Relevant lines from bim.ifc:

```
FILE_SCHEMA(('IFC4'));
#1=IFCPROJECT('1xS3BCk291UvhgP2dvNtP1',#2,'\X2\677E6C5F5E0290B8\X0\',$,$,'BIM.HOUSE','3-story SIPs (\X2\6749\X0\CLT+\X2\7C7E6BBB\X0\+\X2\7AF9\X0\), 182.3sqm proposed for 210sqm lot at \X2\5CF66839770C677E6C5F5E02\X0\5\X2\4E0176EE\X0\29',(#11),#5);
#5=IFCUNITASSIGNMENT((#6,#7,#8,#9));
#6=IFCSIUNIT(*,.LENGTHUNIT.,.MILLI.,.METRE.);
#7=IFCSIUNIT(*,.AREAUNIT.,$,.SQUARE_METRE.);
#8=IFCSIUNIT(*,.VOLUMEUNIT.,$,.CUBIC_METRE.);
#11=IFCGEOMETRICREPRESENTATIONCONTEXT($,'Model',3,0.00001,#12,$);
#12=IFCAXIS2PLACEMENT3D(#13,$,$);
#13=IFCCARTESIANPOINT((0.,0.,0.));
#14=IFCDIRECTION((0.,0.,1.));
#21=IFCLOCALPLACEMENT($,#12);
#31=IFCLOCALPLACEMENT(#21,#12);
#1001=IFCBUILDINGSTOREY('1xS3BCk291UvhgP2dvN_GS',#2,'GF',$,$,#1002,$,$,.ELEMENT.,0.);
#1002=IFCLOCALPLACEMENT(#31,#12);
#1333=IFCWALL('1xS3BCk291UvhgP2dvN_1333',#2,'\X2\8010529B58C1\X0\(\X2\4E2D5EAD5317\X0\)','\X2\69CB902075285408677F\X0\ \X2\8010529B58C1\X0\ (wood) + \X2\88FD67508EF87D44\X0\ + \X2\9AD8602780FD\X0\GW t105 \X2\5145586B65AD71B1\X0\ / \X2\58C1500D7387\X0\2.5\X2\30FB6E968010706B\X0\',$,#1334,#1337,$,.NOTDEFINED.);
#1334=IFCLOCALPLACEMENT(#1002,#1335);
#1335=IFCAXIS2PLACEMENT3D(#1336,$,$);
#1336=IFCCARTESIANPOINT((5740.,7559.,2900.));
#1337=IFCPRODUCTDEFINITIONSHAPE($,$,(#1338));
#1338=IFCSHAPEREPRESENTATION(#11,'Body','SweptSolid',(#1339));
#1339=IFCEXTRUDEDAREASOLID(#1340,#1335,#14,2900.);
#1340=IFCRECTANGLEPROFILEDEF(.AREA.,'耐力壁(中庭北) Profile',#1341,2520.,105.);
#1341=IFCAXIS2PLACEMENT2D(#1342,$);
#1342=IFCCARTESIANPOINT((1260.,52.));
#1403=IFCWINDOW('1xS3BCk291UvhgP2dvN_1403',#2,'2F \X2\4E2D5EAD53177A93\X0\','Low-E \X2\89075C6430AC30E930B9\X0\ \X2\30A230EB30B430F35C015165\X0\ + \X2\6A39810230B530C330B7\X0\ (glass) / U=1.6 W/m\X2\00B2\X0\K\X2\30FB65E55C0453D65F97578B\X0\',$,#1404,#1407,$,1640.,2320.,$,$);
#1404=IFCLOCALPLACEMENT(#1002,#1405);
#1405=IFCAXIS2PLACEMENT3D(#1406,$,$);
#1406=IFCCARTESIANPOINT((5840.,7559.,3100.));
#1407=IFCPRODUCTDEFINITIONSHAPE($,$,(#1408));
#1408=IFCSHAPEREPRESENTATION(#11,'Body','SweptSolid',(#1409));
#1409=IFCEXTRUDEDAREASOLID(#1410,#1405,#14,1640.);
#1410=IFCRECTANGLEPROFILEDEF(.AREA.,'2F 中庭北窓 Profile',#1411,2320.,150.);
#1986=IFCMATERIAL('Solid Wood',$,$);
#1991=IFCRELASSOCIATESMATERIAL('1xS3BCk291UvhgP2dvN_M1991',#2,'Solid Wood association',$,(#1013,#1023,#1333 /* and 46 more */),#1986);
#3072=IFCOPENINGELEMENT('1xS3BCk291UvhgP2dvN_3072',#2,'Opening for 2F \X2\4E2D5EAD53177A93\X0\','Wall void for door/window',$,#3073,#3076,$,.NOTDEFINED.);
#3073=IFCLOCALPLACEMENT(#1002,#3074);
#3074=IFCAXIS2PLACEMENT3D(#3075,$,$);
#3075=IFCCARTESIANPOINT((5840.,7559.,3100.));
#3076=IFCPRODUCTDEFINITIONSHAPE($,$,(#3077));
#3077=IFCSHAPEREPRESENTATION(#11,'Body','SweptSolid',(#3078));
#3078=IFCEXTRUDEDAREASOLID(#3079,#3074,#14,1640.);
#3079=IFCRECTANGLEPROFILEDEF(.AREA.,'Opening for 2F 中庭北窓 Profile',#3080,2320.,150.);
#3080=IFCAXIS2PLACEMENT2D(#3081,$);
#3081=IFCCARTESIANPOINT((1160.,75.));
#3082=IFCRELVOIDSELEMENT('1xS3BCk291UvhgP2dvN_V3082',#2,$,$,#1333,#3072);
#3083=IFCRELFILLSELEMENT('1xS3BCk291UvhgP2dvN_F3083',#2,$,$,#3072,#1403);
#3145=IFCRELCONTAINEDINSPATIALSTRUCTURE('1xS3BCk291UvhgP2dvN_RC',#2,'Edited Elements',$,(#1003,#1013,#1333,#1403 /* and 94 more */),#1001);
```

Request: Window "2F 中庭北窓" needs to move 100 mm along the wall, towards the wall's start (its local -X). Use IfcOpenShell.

```python
import ifcopenshell
import ifcopenshell.api.geometry
import ifcopenshell.util.placement

model = ifcopenshell.open("bim.ifc")

window = model.by_guid("1xS3BCk291UvhgP2dvN_1403")
opening = window.FillsVoids[0].RelatingOpeningElement
wall = opening.VoidsElements[0].RelatingBuildingElement

wall_matrix = ifcopenshell.util.placement.get_local_placement(wall.ObjectPlacement)
shift = wall_matrix[:3, 0] * -100.0
before = ifcopenshell.util.placement.get_local_placement(window.ObjectPlacement)[:3, 3].copy()

# The window is not placed relative to its opening, so move both.
for product in (opening, window):
    matrix = ifcopenshell.util.placement.get_local_placement(product.ObjectPlacement)
    matrix[:3, 3] += shift
    ifcopenshell.api.geometry.edit_object_placement(model, product=product, matrix=matrix, is_si=False)

after = ifcopenshell.util.placement.get_local_placement(window.ObjectPlacement)[:3, 3]
print("window moved by", (after - before).round(3) + 0.0)

model.write("bim_edited.ifc")
```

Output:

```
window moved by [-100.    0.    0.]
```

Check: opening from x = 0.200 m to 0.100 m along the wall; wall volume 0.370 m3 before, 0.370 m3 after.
